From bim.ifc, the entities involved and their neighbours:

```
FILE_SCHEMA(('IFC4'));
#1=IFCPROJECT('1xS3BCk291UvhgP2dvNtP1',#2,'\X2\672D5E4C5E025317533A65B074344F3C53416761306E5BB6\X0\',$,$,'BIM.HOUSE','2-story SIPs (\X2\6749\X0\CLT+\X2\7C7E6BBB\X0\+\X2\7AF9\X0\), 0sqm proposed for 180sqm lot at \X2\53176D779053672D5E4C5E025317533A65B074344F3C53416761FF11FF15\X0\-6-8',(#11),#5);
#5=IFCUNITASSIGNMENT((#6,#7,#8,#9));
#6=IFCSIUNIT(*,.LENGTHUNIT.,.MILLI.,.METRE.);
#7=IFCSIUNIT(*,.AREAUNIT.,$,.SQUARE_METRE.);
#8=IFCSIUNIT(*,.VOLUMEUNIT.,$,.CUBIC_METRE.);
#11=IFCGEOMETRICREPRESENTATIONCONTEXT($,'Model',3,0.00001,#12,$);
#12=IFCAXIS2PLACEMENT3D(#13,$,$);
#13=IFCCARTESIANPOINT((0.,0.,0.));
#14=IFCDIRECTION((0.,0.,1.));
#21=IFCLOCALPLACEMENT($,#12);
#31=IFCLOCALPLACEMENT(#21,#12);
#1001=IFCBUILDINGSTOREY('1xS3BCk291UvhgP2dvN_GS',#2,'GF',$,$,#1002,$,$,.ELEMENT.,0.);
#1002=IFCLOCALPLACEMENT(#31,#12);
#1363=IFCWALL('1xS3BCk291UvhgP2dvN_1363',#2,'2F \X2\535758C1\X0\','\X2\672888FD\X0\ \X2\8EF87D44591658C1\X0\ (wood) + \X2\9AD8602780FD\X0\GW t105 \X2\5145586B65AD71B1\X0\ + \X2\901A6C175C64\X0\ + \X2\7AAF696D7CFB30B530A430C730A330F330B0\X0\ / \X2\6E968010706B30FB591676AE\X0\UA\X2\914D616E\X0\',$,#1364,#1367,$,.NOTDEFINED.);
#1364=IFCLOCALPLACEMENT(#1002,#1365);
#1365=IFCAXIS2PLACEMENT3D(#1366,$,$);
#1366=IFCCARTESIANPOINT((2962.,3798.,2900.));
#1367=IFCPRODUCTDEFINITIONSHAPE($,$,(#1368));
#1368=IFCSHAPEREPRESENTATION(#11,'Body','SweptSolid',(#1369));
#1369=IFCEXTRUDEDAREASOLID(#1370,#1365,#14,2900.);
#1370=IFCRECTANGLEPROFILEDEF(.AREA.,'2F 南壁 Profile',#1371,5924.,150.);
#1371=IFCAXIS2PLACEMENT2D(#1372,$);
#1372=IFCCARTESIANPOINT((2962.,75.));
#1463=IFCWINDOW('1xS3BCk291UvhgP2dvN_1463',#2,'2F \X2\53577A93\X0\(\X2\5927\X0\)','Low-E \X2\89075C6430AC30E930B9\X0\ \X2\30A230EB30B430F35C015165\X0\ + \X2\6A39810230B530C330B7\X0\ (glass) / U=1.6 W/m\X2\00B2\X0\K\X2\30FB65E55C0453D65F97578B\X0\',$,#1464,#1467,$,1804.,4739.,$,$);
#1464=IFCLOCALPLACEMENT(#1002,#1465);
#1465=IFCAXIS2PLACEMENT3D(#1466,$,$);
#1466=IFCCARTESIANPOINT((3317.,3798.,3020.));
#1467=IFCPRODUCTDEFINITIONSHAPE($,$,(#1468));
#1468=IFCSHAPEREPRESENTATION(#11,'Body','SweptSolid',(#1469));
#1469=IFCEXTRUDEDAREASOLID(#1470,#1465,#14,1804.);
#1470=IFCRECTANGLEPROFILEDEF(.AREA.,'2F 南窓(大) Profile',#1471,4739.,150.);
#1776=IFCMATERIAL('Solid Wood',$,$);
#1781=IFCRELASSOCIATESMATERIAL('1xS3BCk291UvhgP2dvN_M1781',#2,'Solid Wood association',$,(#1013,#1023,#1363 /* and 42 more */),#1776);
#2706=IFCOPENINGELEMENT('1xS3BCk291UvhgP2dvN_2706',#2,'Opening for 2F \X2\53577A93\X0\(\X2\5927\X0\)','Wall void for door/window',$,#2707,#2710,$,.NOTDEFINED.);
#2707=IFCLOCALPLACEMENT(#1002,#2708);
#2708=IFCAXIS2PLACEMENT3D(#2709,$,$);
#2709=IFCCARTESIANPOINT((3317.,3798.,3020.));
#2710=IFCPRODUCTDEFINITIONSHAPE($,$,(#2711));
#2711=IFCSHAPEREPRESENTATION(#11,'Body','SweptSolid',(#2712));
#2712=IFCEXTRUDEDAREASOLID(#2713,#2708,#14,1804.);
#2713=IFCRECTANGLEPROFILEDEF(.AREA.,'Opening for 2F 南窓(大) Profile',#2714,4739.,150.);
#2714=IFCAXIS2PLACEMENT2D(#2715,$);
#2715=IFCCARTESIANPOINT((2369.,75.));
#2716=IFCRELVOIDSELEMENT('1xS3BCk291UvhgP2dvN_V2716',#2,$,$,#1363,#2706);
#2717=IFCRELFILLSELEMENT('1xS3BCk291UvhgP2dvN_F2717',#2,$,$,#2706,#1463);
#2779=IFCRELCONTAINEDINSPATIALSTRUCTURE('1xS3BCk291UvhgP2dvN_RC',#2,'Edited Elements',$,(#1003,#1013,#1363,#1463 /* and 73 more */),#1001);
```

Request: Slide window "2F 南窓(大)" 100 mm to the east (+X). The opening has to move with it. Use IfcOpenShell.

```python
import ifcopenshell
import ifcopenshell.api.geometry
import ifcopenshell.util.placement

model = ifcopenshell.open("bim.ifc")

window = model.by_guid("1xS3BCk291UvhgP2dvN_1463")
opening = window.FillsVoids[0].RelatingOpeningElement
wall = opening.VoidsElements[0].RelatingBuildingElement

wall_matrix = ifcopenshell.util.placement.get_local_placement(wall.ObjectPlacement)
shift = wall_matrix[:3, 0] * 100.0
before = ifcopenshell.util.placement.get_local_placement(window.ObjectPlacement)[:3, 3].copy()

# The window is not placed relative to its opening, so move both.
for product in (opening, window):
    matrix = ifcopenshell.util.placement.get_local_placement(product.ObjectPlacement)
    matrix[:3, 3] += shift
    ifcopenshell.api.geometry.edit_object_placement(model, product=product, matrix=matrix, is_si=False)

after = ifcopenshell.util.placement.get_local_placement(window.ObjectPlacement)[:3, 3]
print("window moved by", (after - before).round(3) + 0.0)

model.write("bim_v2.ifc")
```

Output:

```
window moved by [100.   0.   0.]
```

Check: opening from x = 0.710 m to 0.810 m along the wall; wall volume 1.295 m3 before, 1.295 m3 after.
